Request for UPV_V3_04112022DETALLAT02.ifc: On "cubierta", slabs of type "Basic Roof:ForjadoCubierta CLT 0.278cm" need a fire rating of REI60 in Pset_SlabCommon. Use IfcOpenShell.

First a look at what the model holds.

```python
import ifcopenshell
import ifcopenshell.util.element

model = ifcopenshell.open("UPV_V3_04112022DETALLAT02.ifc")
print(model.schema)
storey = next(s for s in model.by_type("IfcBuildingStorey") if s.Name == "cubierta")
slabs = [e for e in ifcopenshell.util.element.get_decomposition(storey) if e.is_a("IfcSlab")]
seen = {}
for e in slabs:
    element_type = ifcopenshell.util.element.get_type(e)
    key = (element_type.Name if element_type != e and element_type else None, ifcopenshell.util.element.get_pset(e, "Pset_SlabCommon", "FireRating"))
    seen[key] = seen.get(key, 0) + 1
for (name, value), count in sorted(seen.items(), key=str):
    print(count, "x", name, "|", value)
```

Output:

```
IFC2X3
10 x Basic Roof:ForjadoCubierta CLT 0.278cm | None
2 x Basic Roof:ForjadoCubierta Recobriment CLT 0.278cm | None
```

```python
import ifcopenshell
import ifcopenshell.api.pset
import ifcopenshell.util.element

model = ifcopenshell.open("UPV_V3_04112022DETALLAT02.ifc")

storey = next(s for s in model.by_type("IfcBuildingStorey") if s.Name == "cubierta")
slabs = [e for e in ifcopenshell.util.element.get_decomposition(storey) if e.is_a("IfcSlab")]

count = 0
for e in slabs:
    element_type = ifcopenshell.util.element.get_type(e)
    if element_type in (None, e) or element_type.Name != "Basic Roof:ForjadoCubierta CLT 0.278cm":
        continue
    # add_pset returns the element's existing set when there is one.
    pset = ifcopenshell.api.pset.add_pset(model, product=e, name="Pset_SlabCommon")
    ifcopenshell.api.pset.edit_pset(model, pset=pset, properties={"FireRating": "REI60"})
    count += 1

print(count, "slabs updated")

model.write("UPV_V3_04112022DETALLAT02_updated.ifc")
```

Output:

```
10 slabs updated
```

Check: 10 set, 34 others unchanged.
